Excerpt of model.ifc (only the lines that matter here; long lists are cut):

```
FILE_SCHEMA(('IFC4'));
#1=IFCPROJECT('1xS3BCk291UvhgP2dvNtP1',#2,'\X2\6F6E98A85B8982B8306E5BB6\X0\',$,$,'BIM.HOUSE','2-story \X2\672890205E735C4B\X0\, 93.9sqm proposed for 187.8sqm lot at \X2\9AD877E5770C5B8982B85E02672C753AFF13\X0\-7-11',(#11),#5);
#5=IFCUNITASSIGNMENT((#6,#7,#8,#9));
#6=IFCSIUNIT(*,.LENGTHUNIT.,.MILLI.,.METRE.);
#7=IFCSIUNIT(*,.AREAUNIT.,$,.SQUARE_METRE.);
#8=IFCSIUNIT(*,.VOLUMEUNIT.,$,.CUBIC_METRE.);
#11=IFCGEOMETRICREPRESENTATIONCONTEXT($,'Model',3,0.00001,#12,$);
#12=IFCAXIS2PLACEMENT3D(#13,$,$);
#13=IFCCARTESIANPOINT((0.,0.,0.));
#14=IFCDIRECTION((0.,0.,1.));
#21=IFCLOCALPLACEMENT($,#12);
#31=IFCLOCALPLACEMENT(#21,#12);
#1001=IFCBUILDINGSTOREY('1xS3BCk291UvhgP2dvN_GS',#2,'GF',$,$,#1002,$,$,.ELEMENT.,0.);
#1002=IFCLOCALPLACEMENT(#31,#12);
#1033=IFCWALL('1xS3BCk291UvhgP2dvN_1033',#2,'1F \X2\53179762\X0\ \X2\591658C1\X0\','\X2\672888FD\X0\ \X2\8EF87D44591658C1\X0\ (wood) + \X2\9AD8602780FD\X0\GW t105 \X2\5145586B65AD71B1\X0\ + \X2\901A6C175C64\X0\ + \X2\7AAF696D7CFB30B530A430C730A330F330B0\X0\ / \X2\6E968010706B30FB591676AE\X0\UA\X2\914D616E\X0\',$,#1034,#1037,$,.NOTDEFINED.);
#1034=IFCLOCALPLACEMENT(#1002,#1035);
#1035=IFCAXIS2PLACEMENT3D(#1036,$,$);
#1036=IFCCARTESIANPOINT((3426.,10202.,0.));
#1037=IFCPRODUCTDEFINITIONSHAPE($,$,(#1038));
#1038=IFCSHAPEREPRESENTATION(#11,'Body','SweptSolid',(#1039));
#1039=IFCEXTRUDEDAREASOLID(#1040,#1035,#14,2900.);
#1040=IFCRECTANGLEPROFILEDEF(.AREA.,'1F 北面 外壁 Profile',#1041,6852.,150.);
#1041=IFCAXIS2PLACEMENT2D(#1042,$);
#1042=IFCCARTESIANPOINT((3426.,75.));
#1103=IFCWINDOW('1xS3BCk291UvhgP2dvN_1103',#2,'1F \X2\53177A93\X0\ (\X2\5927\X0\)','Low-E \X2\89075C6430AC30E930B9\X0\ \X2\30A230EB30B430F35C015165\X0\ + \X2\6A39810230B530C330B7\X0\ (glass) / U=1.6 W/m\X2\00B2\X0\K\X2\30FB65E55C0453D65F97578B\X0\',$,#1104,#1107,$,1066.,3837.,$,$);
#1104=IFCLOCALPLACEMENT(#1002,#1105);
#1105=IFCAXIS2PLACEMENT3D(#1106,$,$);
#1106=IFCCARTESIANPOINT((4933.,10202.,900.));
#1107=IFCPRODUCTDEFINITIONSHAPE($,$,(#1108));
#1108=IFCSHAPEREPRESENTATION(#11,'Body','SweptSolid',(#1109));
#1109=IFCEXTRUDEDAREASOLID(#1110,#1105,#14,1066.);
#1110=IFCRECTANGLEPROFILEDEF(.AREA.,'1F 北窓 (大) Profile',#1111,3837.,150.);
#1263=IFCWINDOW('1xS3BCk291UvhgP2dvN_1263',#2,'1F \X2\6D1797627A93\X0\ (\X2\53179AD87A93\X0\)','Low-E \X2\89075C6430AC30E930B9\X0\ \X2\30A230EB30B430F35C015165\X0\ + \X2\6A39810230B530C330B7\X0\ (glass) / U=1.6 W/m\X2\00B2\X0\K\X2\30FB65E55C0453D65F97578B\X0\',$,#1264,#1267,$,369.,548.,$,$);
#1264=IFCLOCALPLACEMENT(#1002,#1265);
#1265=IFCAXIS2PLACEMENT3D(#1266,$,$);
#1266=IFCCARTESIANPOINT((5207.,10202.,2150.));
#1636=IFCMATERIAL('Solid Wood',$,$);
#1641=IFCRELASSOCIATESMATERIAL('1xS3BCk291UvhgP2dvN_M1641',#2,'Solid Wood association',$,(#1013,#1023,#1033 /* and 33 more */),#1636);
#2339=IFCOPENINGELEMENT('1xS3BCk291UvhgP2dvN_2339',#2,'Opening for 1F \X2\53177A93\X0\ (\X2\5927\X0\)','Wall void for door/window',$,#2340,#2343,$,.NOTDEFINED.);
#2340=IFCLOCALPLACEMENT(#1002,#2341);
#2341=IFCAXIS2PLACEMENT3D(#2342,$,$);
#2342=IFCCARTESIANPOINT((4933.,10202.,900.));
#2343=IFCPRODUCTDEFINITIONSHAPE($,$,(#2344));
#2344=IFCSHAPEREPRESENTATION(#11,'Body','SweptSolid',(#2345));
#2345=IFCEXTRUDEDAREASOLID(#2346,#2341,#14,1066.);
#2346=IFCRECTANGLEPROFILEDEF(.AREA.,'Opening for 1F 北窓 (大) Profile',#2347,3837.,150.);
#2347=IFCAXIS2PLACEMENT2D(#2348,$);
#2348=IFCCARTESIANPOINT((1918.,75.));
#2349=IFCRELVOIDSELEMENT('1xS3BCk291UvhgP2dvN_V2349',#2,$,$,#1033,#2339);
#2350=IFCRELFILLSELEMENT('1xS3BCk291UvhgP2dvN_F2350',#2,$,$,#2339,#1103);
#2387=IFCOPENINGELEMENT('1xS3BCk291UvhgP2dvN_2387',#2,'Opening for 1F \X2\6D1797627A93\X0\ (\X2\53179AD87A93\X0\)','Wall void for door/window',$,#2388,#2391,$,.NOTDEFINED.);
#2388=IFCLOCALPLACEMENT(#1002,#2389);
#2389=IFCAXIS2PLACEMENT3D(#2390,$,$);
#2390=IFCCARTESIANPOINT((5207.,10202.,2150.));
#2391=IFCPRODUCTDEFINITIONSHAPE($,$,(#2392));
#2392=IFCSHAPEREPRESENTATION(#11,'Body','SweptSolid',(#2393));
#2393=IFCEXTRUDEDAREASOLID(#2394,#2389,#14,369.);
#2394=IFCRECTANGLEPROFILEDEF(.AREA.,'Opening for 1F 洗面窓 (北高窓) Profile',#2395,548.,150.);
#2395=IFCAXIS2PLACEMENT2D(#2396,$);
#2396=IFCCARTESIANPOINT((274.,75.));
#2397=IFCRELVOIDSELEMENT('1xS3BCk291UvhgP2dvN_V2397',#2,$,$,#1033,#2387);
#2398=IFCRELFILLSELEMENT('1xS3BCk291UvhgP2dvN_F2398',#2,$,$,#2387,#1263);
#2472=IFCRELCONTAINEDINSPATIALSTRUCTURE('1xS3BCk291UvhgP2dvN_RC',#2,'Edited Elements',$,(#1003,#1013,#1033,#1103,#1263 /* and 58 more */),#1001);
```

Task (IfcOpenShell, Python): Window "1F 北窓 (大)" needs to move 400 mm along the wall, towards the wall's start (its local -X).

```python
import ifcopenshell
import ifcopenshell.api.geometry
import ifcopenshell.util.placement
import ifcopenshell.util.unit

model = ifcopenshell.open("model.ifc")
unit_scale = ifcopenshell.util.unit.calculate_unit_scale(model)

window = model.by_guid("1xS3BCk291UvhgP2dvN_1103")
opening = window.FillsVoids[0].RelatingOpeningElement
wall = opening.VoidsElements[0].RelatingBuildingElement

wall_matrix = ifcopenshell.util.placement.get_local_placement(wall.ObjectPlacement)
shift = wall_matrix[:3, 0] * -0.4 / unit_scale
before = ifcopenshell.util.placement.get_local_placement(window.ObjectPlacement)[:3, 3].copy()

# The window is not placed relative to its opening, so move both.
for product in (opening, window):
    matrix = ifcopenshell.util.placement.get_local_placement(product.ObjectPlacement)
    matrix[:3, 3] += shift
    ifcopenshell.api.geometry.edit_object_placement(model, product=product, matrix=matrix, is_si=False)

after = ifcopenshell.util.placement.get_local_placement(window.ObjectPlacement)[:3, 3]
print("window moved by", (after - before).round(3) + 0.0)

model.write("model_edited.ifc")
```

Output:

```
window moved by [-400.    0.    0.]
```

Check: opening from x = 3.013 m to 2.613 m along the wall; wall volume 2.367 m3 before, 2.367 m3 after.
